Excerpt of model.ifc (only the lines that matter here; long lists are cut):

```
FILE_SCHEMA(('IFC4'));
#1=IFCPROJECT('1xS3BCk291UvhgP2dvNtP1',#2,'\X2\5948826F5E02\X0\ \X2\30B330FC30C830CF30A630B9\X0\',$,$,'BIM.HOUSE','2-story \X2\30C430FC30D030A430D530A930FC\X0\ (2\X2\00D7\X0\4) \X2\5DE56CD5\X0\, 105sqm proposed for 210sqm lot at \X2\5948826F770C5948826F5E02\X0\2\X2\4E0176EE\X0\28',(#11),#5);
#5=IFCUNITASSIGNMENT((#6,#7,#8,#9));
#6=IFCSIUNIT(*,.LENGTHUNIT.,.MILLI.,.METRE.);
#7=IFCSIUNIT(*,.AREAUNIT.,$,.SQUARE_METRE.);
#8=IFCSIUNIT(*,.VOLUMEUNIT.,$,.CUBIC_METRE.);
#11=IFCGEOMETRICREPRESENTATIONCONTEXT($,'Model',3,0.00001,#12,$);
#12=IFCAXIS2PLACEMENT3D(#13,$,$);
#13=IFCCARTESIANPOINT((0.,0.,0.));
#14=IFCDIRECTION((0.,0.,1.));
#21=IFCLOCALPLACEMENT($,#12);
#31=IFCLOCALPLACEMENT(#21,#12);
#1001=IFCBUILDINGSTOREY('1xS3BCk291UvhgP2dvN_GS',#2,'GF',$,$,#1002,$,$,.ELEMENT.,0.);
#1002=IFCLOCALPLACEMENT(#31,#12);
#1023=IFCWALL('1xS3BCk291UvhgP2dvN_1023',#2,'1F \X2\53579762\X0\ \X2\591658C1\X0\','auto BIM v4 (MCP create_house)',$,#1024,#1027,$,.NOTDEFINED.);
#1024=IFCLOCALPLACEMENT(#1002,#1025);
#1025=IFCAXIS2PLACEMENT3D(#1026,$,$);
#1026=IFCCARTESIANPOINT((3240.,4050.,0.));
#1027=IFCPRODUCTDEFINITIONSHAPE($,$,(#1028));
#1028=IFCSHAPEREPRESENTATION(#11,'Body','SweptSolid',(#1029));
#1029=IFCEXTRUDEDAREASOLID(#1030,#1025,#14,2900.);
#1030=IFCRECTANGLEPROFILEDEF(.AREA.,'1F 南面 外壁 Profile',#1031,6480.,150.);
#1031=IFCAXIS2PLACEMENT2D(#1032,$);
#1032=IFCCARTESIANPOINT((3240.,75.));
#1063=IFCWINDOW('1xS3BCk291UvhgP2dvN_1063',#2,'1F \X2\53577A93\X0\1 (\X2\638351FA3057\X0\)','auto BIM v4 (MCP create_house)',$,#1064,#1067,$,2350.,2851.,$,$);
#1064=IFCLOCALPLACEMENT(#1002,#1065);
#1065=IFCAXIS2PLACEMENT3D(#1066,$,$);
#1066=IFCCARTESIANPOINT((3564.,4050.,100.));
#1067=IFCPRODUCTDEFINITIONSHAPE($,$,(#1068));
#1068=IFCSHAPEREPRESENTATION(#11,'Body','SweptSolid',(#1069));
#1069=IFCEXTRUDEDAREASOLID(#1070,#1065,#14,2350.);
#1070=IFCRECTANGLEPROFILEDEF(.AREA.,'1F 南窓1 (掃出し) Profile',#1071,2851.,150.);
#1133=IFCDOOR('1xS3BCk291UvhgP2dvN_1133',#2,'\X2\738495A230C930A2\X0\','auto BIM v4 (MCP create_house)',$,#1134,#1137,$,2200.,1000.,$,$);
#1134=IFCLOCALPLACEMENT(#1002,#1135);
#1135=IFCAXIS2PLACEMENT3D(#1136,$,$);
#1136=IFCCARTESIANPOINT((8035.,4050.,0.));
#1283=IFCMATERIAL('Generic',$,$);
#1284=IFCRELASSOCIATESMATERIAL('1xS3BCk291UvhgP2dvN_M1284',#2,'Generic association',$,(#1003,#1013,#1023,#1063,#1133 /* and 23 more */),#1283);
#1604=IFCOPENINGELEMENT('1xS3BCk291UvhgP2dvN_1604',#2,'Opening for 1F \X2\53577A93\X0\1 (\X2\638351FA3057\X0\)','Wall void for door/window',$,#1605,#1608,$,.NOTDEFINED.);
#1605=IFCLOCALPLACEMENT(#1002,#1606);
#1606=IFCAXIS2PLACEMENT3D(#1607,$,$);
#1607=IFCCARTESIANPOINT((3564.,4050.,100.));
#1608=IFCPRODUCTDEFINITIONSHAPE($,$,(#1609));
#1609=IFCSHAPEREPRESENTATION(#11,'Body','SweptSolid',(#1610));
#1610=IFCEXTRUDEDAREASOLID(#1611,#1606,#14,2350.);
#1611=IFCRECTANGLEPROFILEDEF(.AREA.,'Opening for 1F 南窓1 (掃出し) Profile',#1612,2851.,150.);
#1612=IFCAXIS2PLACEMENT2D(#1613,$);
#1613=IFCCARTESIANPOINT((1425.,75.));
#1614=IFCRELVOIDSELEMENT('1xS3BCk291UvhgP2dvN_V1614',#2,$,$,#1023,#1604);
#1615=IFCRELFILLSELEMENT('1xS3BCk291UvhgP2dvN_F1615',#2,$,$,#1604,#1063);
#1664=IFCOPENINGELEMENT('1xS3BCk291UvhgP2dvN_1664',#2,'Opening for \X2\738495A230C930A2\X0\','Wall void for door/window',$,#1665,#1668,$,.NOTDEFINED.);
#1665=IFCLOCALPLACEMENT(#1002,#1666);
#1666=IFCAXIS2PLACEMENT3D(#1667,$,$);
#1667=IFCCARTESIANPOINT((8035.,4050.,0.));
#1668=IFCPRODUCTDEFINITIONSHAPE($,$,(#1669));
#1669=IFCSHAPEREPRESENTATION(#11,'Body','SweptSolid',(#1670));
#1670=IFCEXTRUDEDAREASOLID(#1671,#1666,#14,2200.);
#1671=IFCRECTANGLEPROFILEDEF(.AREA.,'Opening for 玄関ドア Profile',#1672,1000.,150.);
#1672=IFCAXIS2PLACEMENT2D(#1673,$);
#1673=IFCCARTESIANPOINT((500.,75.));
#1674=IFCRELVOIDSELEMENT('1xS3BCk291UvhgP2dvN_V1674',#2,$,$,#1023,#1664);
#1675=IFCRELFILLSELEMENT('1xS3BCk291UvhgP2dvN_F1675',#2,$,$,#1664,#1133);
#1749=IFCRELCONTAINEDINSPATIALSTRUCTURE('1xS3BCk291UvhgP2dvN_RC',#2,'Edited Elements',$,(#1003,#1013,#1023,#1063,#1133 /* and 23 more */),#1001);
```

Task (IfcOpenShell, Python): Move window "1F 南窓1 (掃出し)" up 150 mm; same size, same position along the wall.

```python
import numpy as np
import ifcopenshell
import ifcopenshell.api.geometry
import ifcopenshell.util.placement
import ifcopenshell.util.unit

model = ifcopenshell.open("model.ifc")
unit_scale = ifcopenshell.util.unit.calculate_unit_scale(model)

window = model.by_guid("1xS3BCk291UvhgP2dvN_1063")
opening = window.FillsVoids[0].RelatingOpeningElement
dz = 150.0

shift = np.array([0.0, 0.0, dz])
# The window is not placed relative to its opening, so move both.
for product in (opening, window):
    matrix = ifcopenshell.util.placement.get_local_placement(product.ObjectPlacement)
    matrix[:3, 3] += shift
    ifcopenshell.api.geometry.edit_object_placement(model, product=product, matrix=matrix, is_si=False)

print(f"moved by {dz * unit_scale:+.3f} m")

model.write("model_v2.ifc")
```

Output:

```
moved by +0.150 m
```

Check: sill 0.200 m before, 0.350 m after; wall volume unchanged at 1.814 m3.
